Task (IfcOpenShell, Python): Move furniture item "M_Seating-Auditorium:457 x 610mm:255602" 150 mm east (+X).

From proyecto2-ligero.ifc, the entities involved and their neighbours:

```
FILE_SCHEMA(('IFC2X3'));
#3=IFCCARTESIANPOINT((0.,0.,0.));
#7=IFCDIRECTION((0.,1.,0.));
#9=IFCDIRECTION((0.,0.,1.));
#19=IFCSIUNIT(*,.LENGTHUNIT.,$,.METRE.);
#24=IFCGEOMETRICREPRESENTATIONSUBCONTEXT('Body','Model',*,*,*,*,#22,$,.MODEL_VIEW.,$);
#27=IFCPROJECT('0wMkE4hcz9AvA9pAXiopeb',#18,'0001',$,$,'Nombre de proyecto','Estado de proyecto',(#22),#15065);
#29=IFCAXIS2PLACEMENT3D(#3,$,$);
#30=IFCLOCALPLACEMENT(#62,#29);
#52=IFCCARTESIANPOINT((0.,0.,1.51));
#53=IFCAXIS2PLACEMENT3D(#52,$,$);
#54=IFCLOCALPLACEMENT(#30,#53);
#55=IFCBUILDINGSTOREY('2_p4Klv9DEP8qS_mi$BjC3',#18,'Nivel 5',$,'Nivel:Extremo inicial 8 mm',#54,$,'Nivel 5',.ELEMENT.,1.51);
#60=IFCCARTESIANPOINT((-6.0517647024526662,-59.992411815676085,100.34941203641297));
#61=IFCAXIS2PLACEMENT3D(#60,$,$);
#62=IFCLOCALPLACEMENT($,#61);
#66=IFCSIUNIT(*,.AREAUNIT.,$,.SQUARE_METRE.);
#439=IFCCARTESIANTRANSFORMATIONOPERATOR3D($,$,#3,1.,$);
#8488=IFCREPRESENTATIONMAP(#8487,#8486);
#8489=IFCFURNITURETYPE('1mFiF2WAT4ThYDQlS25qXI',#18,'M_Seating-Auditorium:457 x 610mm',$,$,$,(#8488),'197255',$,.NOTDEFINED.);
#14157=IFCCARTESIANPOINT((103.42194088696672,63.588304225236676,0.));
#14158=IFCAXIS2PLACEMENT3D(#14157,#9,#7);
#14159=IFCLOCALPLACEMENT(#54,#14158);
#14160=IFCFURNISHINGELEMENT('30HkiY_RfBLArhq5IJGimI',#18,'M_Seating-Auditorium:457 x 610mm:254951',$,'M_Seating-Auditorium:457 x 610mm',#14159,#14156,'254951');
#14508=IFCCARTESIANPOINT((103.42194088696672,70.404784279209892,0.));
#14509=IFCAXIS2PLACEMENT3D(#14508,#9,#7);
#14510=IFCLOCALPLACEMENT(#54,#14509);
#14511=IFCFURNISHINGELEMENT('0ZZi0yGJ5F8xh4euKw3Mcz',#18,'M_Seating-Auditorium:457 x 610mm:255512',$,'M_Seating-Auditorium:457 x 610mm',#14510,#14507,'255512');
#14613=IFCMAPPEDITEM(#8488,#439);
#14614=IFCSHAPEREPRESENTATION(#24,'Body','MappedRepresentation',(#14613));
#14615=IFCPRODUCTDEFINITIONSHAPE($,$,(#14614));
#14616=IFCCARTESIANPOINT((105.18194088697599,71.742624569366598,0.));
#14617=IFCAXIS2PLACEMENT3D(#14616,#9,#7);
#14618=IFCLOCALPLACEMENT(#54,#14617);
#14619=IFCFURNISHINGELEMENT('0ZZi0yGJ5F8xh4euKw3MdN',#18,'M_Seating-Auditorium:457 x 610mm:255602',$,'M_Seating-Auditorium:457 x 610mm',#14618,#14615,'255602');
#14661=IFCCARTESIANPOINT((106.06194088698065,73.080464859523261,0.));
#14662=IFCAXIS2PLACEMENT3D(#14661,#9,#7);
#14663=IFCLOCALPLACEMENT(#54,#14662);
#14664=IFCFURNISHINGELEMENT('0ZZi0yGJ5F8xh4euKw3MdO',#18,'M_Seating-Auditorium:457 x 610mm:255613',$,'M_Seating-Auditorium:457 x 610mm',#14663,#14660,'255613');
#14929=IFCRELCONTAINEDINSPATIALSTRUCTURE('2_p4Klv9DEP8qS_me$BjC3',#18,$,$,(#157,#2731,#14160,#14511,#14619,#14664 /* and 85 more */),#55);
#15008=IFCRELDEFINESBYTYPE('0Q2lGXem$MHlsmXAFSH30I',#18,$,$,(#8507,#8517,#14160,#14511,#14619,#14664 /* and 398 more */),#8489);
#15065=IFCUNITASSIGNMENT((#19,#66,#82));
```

```python
import ifcopenshell
import ifcopenshell.api.geometry
import ifcopenshell.util.placement
import ifcopenshell.util.unit

model = ifcopenshell.open("proyecto2-ligero.ifc")
unit_scale = ifcopenshell.util.unit.calculate_unit_scale(model)

item = model.by_guid("0ZZi0yGJ5F8xh4euKw3MdN")
matrix = ifcopenshell.util.placement.get_local_placement(item.ObjectPlacement)
matrix[0, 3] += 0.15 / unit_scale
ifcopenshell.api.geometry.edit_object_placement(model, product=item, matrix=matrix, is_si=False)

print(ifcopenshell.util.placement.get_local_placement(item.ObjectPlacement).round(3) + 0.0)

model.write("proyecto2-ligero-out.ifc")
```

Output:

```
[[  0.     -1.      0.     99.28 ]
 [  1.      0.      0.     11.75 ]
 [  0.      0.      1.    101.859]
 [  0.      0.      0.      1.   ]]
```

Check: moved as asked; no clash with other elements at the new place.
